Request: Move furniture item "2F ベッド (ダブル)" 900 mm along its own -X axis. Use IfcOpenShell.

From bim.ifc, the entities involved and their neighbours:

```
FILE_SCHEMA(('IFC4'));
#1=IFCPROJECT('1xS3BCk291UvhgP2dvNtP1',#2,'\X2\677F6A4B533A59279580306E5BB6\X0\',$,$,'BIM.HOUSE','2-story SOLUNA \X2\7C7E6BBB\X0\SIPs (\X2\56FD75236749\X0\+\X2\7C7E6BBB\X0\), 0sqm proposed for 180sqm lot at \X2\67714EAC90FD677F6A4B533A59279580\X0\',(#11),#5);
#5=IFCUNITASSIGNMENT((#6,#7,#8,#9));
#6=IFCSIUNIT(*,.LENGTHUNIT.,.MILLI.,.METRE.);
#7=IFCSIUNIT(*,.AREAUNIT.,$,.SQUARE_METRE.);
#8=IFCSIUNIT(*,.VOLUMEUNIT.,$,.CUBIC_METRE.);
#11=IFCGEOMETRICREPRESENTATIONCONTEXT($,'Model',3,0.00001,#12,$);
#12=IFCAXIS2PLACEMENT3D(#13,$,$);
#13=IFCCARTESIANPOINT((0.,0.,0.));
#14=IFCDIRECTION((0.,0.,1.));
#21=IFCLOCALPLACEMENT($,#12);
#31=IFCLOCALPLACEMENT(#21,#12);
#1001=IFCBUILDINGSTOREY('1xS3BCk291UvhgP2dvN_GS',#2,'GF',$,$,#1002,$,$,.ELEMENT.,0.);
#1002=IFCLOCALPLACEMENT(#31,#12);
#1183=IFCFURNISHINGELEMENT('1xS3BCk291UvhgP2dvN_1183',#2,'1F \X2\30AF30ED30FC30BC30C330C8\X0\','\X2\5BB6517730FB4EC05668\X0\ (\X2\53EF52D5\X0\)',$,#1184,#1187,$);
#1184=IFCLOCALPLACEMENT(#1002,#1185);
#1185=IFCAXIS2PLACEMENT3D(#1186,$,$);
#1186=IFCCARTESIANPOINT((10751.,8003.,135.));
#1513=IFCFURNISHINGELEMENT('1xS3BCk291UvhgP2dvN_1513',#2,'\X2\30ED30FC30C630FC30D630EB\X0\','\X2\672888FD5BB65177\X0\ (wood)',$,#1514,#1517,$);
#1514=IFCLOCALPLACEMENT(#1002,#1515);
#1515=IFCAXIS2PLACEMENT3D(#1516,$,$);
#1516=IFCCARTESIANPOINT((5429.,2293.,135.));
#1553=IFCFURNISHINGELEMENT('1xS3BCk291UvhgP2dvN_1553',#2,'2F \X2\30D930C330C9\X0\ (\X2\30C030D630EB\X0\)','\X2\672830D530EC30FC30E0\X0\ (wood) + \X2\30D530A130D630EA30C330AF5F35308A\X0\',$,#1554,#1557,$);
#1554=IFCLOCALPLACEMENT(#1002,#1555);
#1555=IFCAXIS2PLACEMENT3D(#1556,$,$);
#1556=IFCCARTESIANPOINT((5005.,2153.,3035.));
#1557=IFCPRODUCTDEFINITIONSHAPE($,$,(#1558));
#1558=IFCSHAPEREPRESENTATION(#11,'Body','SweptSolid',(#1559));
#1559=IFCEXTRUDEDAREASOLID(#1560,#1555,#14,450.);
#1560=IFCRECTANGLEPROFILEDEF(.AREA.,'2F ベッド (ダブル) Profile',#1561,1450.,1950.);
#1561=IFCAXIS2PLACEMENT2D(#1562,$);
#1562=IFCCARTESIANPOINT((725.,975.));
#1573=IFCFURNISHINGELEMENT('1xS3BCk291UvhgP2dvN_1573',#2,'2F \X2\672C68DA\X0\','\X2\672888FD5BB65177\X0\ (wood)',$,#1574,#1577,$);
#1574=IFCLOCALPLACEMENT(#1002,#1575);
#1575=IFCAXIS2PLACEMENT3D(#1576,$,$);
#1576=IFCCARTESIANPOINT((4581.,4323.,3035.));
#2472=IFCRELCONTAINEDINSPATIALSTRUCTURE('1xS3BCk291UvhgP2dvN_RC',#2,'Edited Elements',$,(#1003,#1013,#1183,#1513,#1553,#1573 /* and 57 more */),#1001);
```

```python
import ifcopenshell
import ifcopenshell.api.geometry
import ifcopenshell.util.placement
import ifcopenshell.util.unit

model = ifcopenshell.open("bim.ifc")
unit_scale = ifcopenshell.util.unit.calculate_unit_scale(model)

item = model.by_guid("1xS3BCk291UvhgP2dvN_1553")
matrix = ifcopenshell.util.placement.get_local_placement(item.ObjectPlacement)
matrix[:3, 3] -= matrix[:3, 0] * 0.9 / unit_scale
ifcopenshell.api.geometry.edit_object_placement(model, product=item, matrix=matrix, is_si=False)

print(ifcopenshell.util.placement.get_local_placement(item.ObjectPlacement).round(3) + 0.0)

model.write("bim_v2.ifc")
```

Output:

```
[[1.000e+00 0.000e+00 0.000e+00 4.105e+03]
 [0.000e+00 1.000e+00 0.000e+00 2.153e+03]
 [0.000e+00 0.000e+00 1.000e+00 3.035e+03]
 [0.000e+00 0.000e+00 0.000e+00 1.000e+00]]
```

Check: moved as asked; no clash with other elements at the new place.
